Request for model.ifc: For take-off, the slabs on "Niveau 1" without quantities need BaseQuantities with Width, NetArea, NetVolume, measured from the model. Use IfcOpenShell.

First a look at what the model holds.

```python
import ifcopenshell
import ifcopenshell.util.element
import ifcopenshell.util.unit

model = ifcopenshell.open("model.ifc")
print(model.schema)
for unit_type in ("LENGTHUNIT", "AREAUNIT", "VOLUMEUNIT"):
    print(unit_type, ifcopenshell.util.unit.calculate_unit_scale(model, unit_type))
storey = next(s for s in model.by_type("IfcBuildingStorey") if s.Name == "Niveau 1")
slabs = [e for e in ifcopenshell.util.element.get_decomposition(storey) if e.is_a("IfcSlab")]
for e in sorted(slabs, key=lambda e: e.id()):
    print(e.id(), e.is_a(), e.Name, list(ifcopenshell.util.element.get_psets(e, qtos_only=True)), sep=" | ")
```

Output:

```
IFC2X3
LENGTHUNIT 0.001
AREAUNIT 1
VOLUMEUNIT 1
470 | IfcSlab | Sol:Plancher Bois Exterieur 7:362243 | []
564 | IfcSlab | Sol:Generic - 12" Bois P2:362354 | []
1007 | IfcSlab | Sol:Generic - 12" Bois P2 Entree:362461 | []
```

```python
import ifcopenshell
import ifcopenshell.api.pset
import ifcopenshell.geom
import ifcopenshell.util.element
import ifcopenshell.util.shape
import ifcopenshell.util.unit

model = ifcopenshell.open("model.ifc")
unit_scale = ifcopenshell.util.unit.calculate_unit_scale(model)
area_scale = ifcopenshell.util.unit.calculate_unit_scale(model, "AREAUNIT")
volume_scale = ifcopenshell.util.unit.calculate_unit_scale(model, "VOLUMEUNIT")
settings = ifcopenshell.geom.settings()

storey = next(s for s in model.by_type("IfcBuildingStorey") if s.Name == "Niveau 1")
slabs = [e for e in ifcopenshell.util.element.get_decomposition(storey) if e.is_a("IfcSlab")]

for e in sorted(slabs, key=lambda e: e.id()):
    if ifcopenshell.util.element.get_psets(e, qtos_only=True, should_inherit=False):
        continue
    # Geometry comes back in metres, in the element's own axes.
    shape = ifcopenshell.geom.create_shape(settings, e)
    values = {
        "Width": ifcopenshell.util.shape.get_z(shape.geometry) / unit_scale,
        "NetArea": ifcopenshell.util.shape.get_footprint_area(shape.geometry) / area_scale,
        "NetVolume": ifcopenshell.util.shape.get_volume(shape.geometry) / volume_scale,
    }
    qto = ifcopenshell.api.pset.add_qto(model, product=e, name="BaseQuantities")
    ifcopenshell.api.pset.edit_qto(model, qto=qto, properties=values)
    print(e.id(), {k: round(v, 3) for k, v in values.items()})

model.write("model-out.ifc")
```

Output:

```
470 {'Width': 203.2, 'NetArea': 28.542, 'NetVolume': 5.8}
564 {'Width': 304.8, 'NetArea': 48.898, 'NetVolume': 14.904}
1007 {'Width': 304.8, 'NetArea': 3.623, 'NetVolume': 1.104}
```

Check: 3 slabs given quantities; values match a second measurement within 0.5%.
